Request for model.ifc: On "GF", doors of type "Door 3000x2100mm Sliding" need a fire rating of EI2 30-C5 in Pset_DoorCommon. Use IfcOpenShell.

First a look at what the model holds.

```python
import ifcopenshell
import ifcopenshell.util.element

model = ifcopenshell.open("model.ifc")
print(model.schema)
storey = next(s for s in model.by_type("IfcBuildingStorey") if s.Name == "GF")
doors = [e for e in ifcopenshell.util.element.get_decomposition(storey) if e.is_a("IfcDoor")]
seen = {}
for e in doors:
    element_type = ifcopenshell.util.element.get_type(e)
    key = (element_type.Name if element_type != e and element_type else None, ifcopenshell.util.element.get_pset(e, "Pset_DoorCommon", "FireRating"))
    seen[key] = seen.get(key, 0) + 1
for (name, value), count in sorted(seen.items(), key=str):
    print(count, "x", name, "|", value)
```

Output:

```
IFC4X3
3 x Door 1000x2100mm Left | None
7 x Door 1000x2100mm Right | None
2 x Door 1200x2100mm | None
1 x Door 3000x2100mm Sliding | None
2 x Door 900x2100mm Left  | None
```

```python
import ifcopenshell
import ifcopenshell.api.pset
import ifcopenshell.util.element

model = ifcopenshell.open("model.ifc")

storey = next(s for s in model.by_type("IfcBuildingStorey") if s.Name == "GF")
doors = [e for e in ifcopenshell.util.element.get_decomposition(storey) if e.is_a("IfcDoor")]

count = 0
for e in doors:
    element_type = ifcopenshell.util.element.get_type(e)
    if element_type in (None, e) or element_type.Name != "Door 3000x2100mm Sliding":
        continue
    # add_pset returns the element's existing set when there is one.
    pset = ifcopenshell.api.pset.add_pset(model, product=e, name="Pset_DoorCommon")
    ifcopenshell.api.pset.edit_pset(model, pset=pset, properties={"FireRating": "EI2 30-C5"})
    count += 1

print(count, "doors updated")

model.write("model_updated.ifc")
```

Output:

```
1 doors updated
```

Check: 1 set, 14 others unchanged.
